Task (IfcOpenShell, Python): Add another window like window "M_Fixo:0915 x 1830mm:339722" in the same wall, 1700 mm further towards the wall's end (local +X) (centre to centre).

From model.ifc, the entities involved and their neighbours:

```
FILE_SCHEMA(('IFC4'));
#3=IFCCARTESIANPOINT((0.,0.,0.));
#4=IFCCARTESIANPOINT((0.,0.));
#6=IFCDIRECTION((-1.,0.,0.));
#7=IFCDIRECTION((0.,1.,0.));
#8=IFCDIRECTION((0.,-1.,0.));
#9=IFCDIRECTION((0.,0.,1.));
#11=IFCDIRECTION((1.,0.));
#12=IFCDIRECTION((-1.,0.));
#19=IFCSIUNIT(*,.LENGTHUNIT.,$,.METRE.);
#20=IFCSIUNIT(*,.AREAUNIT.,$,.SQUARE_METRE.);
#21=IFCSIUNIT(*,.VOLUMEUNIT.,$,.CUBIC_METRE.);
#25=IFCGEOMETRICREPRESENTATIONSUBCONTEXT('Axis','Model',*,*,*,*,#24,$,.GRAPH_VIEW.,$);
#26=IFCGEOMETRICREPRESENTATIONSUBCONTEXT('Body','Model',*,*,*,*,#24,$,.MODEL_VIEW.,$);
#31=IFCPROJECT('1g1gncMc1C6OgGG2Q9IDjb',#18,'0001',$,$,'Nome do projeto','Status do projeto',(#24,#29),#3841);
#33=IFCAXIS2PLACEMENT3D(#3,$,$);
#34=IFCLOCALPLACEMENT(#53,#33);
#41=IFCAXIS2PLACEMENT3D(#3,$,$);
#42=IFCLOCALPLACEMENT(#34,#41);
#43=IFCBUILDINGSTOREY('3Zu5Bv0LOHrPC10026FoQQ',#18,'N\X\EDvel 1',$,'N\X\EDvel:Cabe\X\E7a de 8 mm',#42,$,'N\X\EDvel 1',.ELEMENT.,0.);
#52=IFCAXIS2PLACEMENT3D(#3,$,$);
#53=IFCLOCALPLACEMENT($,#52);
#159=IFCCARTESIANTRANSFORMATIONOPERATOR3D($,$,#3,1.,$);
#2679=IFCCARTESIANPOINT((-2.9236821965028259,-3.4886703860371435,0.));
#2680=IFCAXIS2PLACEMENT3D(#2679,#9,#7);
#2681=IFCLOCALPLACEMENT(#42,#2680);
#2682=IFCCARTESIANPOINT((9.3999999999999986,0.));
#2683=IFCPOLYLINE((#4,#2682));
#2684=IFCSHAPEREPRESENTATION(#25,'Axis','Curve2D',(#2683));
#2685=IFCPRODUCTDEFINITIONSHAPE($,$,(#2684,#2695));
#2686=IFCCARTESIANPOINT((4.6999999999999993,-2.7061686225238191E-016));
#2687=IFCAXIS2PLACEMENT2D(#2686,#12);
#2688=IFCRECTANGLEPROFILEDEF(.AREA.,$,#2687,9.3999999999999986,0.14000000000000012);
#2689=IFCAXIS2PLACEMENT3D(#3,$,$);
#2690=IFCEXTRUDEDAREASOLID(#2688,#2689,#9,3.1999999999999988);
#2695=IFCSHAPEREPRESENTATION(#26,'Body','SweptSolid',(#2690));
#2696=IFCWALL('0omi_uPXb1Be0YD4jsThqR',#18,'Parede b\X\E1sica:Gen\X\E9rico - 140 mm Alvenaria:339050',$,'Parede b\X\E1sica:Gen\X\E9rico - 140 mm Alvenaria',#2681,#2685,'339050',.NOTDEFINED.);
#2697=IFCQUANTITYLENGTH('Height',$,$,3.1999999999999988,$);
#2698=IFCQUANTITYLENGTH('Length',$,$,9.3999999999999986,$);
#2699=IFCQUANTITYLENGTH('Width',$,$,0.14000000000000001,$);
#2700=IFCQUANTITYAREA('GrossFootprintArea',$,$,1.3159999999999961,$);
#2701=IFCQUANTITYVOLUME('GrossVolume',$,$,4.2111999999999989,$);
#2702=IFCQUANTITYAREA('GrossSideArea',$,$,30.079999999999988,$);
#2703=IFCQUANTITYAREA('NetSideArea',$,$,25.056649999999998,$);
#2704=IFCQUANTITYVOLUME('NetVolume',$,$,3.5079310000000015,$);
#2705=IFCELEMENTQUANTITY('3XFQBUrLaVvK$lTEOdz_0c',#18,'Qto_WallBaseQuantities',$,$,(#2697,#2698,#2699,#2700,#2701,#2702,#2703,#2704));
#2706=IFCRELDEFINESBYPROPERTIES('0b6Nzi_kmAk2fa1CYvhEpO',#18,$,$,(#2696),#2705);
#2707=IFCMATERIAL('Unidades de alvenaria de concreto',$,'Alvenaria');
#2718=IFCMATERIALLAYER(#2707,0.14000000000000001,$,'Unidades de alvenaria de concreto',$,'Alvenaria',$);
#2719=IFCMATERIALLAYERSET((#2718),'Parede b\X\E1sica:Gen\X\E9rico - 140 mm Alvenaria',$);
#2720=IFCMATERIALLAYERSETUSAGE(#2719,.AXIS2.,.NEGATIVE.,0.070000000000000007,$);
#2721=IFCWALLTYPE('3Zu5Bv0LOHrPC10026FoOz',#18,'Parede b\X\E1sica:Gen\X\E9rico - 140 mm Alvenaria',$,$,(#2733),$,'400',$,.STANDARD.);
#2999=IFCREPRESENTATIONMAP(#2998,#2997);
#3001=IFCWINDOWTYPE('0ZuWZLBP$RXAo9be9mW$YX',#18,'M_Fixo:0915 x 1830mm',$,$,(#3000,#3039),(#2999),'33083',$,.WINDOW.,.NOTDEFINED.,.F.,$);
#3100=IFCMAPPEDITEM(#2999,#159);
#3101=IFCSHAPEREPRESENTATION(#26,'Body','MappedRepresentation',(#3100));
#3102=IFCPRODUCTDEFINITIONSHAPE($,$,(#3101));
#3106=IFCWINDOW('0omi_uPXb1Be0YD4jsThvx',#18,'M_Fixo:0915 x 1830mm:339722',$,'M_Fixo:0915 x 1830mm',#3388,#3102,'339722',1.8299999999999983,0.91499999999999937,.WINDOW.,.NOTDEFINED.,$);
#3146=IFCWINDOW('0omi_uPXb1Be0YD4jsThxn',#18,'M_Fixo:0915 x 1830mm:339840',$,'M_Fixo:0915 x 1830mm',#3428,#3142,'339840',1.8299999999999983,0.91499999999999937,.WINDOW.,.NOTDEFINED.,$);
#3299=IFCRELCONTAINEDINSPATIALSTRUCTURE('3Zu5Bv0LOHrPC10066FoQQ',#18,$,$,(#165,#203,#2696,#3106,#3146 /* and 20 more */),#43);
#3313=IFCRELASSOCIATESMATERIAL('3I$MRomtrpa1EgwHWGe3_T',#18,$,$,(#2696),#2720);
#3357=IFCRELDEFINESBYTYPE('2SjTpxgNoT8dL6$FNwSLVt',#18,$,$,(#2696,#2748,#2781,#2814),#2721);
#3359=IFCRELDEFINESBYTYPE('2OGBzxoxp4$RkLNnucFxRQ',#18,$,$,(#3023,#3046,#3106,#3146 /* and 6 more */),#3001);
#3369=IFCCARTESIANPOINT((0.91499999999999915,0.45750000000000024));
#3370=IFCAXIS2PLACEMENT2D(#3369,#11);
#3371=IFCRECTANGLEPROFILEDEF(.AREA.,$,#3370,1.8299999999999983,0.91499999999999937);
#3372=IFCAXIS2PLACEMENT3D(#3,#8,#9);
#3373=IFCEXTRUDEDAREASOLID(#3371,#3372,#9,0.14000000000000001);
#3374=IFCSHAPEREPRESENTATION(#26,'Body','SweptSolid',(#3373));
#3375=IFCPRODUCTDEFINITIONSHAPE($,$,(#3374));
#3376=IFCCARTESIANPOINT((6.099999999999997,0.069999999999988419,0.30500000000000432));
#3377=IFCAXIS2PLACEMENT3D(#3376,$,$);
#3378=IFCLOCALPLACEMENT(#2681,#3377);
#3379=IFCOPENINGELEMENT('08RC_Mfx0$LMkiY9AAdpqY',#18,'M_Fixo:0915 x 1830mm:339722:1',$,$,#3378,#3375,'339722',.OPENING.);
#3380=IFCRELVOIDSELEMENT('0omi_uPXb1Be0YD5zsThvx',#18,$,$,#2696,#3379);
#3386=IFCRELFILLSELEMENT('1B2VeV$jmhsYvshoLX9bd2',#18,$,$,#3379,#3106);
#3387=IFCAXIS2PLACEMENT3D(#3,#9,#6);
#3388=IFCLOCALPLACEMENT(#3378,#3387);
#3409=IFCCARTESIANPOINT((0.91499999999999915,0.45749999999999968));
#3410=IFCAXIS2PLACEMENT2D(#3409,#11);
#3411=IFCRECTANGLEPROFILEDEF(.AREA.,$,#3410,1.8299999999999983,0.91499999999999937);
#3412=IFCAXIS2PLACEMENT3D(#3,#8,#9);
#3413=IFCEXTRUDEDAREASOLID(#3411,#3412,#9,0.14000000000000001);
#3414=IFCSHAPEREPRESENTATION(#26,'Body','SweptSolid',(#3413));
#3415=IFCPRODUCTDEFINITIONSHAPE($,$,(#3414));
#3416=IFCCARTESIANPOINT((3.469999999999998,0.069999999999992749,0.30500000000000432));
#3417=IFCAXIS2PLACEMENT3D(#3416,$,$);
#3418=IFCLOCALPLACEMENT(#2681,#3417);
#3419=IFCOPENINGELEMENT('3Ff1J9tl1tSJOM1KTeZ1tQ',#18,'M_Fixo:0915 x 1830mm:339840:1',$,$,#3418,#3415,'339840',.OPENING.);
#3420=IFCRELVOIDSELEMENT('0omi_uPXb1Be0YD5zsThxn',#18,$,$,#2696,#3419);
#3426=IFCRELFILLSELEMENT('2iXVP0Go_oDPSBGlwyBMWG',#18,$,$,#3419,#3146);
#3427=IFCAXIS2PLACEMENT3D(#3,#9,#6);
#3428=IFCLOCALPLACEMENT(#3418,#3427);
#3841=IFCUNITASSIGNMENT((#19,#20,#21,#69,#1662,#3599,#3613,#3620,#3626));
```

```python
import ifcopenshell
import ifcopenshell.api.feature
import ifcopenshell.api.geometry
import ifcopenshell.api.pset
import ifcopenshell.api.root
import ifcopenshell.geom
import ifcopenshell.util.element
import ifcopenshell.util.placement
import ifcopenshell.util.shape
import ifcopenshell.util.unit

model = ifcopenshell.open("model.ifc")
unit_scale = ifcopenshell.util.unit.calculate_unit_scale(model)
area_scale = ifcopenshell.util.unit.calculate_unit_scale(model, "AREAUNIT")
volume_scale = ifcopenshell.util.unit.calculate_unit_scale(model, "VOLUMEUNIT")
settings = ifcopenshell.geom.settings()


def volume(element):
    """Net volume in cubic metres, openings subtracted."""
    shape = ifcopenshell.geom.create_shape(settings, element)
    return ifcopenshell.util.shape.get_volume(shape.geometry)


def reuse_history(source, copy):
    """copy_class also copies each property set's owner history, people and application; keep the originals."""
    for rel in copy.IsDefinedBy:
        if rel.is_a("IfcRelDefinesByProperties") and (history := rel.RelatingPropertyDefinition.OwnerHistory):
            rel.RelatingPropertyDefinition.OwnerHistory = source.OwnerHistory
            ifcopenshell.util.element.remove_deep2(model, history)


window = model.by_guid("0omi_uPXb1Be0YD4jsThvx")
opening = window.FillsVoids[0].RelatingOpeningElement
wall = opening.VoidsElements[0].RelatingBuildingElement
before = volume(wall)
shift = ifcopenshell.util.placement.get_local_placement(wall.ObjectPlacement)[:3, 0] * 1.7 / unit_scale

# copy_class copies the void relationship, type, container and properties, but no geometry.
new_opening = ifcopenshell.api.root.copy_class(model, product=opening)
new_opening.Representation = ifcopenshell.util.element.copy_deep(
    model, opening.Representation, exclude=["IfcGeometricRepresentationContext", "IfcRepresentationMap"]
)
new_opening.Name = "M_Fixo:0915 x 1830mm"
new_opening.Tag = None
reuse_history(opening, new_opening)
new_window = ifcopenshell.api.root.copy_class(model, product=window)
new_window.Representation = ifcopenshell.util.element.copy_deep(
    model, window.Representation, exclude=["IfcGeometricRepresentationContext", "IfcRepresentationMap"]
)
new_window.Name = "M_Fixo:0915 x 1830mm"
new_window.Tag = None
reuse_history(window, new_window)
ifcopenshell.api.feature.add_filling(model, opening=new_opening, element=new_window)

for old, new in ((opening, new_opening), (window, new_window)):
    matrix = ifcopenshell.util.placement.get_local_placement(old.ObjectPlacement)
    matrix[:3, 3] += shift
    ifcopenshell.api.geometry.edit_object_placement(model, product=new, matrix=matrix, is_si=False)

after = volume(wall)
thickness = 0.14  # wall thickness in metres

# Update the wall's stored quantities.
qto = model.by_id(ifcopenshell.util.element.get_pset(wall, "Qto_WallBaseQuantities", should_inherit=False)["id"])
ifcopenshell.api.pset.edit_qto(model, qto=qto, properties={
    "NetSideArea": after / thickness / area_scale,
    "NetVolume": after / volume_scale,
})

print(f"wall volume {before:.3f} -> {after:.3f} m3")

model.write("model_rev.ifc")
```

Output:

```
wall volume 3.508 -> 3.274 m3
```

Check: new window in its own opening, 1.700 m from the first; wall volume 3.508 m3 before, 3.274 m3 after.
